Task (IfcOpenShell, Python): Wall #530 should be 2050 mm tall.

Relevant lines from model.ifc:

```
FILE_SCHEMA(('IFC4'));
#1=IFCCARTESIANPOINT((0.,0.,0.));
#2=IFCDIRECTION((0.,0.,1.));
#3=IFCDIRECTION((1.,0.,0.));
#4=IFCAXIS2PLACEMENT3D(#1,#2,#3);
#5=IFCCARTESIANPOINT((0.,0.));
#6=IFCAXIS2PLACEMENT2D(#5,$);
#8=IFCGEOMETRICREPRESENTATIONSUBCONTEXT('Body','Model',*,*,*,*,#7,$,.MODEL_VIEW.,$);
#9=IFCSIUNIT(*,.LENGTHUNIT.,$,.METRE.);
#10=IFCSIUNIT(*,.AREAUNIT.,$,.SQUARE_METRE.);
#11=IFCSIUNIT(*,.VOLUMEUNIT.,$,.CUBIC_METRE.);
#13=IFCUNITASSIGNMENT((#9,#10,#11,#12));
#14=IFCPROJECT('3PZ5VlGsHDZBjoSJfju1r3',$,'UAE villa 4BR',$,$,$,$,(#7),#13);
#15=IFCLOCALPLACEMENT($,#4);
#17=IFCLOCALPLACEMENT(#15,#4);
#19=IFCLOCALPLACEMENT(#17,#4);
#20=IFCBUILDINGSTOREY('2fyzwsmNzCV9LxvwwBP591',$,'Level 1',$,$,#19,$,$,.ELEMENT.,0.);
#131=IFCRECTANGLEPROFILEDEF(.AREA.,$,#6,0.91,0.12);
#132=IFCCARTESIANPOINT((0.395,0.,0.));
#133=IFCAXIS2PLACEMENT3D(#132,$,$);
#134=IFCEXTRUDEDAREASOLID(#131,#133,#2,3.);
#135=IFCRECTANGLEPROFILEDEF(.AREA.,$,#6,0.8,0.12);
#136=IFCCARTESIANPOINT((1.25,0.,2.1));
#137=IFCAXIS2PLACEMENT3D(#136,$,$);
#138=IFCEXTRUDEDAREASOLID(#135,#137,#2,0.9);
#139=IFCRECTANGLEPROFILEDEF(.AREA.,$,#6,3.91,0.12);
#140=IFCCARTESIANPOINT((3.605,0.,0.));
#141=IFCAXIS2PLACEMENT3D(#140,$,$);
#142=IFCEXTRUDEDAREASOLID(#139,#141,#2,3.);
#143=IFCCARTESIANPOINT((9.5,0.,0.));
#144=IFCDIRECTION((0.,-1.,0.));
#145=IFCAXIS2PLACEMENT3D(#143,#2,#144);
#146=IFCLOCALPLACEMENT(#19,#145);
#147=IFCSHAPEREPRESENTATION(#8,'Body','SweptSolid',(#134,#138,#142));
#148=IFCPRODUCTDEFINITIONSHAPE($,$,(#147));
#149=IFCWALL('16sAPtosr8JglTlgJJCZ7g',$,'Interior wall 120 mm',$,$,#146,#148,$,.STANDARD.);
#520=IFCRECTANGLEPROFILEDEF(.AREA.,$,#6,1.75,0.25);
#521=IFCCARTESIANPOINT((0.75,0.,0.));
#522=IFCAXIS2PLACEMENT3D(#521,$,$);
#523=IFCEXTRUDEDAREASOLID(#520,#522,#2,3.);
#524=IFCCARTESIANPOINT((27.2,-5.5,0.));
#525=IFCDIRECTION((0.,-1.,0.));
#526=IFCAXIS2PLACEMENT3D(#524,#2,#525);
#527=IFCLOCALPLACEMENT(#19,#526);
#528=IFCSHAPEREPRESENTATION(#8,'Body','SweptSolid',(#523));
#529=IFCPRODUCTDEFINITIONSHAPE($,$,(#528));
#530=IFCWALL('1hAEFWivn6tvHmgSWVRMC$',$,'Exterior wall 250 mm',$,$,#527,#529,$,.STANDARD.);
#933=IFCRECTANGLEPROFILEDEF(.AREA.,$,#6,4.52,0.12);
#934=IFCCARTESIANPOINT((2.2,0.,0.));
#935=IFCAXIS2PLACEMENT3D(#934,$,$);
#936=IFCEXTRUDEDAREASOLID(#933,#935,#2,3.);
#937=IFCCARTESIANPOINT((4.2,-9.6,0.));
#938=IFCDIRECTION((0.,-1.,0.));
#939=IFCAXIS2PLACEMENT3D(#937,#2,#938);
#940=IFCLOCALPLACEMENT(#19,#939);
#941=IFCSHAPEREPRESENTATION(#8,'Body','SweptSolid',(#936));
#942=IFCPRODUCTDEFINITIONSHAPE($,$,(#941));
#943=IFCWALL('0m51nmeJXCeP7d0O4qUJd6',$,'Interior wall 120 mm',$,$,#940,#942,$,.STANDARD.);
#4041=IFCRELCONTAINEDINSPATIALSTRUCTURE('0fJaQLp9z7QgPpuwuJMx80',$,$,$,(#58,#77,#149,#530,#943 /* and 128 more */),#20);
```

```python
import ifcopenshell
import ifcopenshell.geom
import ifcopenshell.util.representation
import ifcopenshell.util.shape

model = ifcopenshell.open("model.ifc")
settings = ifcopenshell.geom.settings()


def volume(element):
    """Net volume in cubic metres, openings subtracted."""
    shape = ifcopenshell.geom.create_shape(settings, element)
    return ifcopenshell.util.shape.get_volume(shape.geometry)


wall = model.by_guid("1hAEFWivn6tvHmgSWVRMC$")
before = volume(wall)

body = ifcopenshell.util.representation.get_representation(wall, "Model", "Body")
solid = body.Items[0]
old_height = solid.Depth
solid.Depth = 2.05
after = volume(wall)

print(f"height {old_height:g} -> {solid.Depth:g}, volume {before:.3f} -> {after:.3f} m3")

model.write("model_updated.ifc")
```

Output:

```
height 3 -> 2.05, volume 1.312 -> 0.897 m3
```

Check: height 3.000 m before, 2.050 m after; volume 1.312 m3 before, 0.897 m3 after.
